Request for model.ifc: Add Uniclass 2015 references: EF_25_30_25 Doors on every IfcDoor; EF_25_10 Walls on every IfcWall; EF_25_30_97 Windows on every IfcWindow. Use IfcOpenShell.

First a look at what the model holds.

```python
import ifcopenshell

model = ifcopenshell.open("model.ifc")
print(model.schema)
print("classifications:", [c.Name for c in model.by_type("IfcClassification")])
for ifc_class in ("IfcDoor", "IfcRoof", "IfcStair", "IfcWall", "IfcWindow"):
    print(ifc_class, len(model.by_type(ifc_class)))
```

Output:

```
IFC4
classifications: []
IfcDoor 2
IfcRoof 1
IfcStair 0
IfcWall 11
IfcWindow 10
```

```python
import ifcopenshell
import ifcopenshell.api.classification

model = ifcopenshell.open("model.ifc")

system = ifcopenshell.api.classification.add_classification(model, classification="Uniclass 2015")

codes = {
    "IfcDoor": ("EF_25_30_25", "Doors"),
    "IfcWall": ("EF_25_10", "Walls"),
    "IfcWindow": ("EF_25_30_97", "Windows"),
}
for ifc_class, (code, name) in codes.items():
    products = model.by_type(ifc_class)
    ifcopenshell.api.classification.add_reference(
        model, products=products, classification=system, identification=code, name=name
    )
    print(code, len(products))

model.write("model_edited.ifc")
```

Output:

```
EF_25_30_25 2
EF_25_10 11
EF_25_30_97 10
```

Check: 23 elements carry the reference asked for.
